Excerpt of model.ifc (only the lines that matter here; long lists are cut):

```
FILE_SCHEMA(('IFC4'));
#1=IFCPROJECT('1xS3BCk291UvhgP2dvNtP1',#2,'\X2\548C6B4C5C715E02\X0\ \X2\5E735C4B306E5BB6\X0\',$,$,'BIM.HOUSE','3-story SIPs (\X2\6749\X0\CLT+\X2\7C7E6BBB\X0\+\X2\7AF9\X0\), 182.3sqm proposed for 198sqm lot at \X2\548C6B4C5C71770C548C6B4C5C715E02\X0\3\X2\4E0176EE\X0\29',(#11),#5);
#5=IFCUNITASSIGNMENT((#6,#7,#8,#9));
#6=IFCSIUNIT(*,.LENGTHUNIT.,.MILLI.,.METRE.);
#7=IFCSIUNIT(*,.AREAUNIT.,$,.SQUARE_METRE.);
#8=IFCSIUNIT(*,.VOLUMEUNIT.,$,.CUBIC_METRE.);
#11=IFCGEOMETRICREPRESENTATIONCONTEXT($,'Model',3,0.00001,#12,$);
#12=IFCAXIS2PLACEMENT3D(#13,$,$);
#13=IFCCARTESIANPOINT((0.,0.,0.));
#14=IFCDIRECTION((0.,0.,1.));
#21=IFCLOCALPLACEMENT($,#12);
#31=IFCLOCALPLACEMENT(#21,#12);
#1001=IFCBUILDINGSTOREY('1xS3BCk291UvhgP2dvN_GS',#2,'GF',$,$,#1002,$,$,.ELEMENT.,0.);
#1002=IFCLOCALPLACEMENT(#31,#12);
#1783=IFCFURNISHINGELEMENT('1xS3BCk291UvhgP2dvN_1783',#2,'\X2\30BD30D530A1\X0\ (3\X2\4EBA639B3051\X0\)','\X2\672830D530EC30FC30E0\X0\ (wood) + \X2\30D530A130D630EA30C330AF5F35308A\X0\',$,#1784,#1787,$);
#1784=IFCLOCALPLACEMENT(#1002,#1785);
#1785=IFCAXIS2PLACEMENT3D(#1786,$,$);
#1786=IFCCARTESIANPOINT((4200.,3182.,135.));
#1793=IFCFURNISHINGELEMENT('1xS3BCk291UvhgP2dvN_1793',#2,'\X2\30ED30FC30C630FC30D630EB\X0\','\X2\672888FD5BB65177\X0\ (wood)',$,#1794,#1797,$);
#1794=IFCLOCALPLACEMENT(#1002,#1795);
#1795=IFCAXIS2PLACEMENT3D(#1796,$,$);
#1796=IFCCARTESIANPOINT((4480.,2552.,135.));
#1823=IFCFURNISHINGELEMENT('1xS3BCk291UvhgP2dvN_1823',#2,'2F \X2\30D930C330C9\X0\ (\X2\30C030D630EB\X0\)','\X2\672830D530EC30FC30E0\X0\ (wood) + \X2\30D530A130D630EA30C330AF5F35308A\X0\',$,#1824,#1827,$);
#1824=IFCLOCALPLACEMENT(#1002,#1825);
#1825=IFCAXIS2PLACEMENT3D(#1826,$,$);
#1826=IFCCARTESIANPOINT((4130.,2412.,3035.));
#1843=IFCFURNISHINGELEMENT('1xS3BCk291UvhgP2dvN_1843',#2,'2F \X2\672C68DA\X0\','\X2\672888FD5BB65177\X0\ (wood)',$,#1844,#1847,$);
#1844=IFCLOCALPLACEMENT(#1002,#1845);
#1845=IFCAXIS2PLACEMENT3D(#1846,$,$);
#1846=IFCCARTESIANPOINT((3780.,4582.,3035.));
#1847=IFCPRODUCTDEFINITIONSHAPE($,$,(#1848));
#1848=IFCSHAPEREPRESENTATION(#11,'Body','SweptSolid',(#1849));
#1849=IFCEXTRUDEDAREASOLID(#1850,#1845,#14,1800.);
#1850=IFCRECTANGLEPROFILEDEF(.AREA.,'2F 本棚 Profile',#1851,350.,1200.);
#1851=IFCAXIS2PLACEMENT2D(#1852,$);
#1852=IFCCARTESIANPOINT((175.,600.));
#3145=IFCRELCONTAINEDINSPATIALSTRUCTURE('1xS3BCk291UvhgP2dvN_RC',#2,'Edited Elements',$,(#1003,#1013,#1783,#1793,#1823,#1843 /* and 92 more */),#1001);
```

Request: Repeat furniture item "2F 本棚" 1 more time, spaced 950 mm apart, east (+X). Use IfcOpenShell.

```python
import numpy as np
import ifcopenshell
import ifcopenshell.api.geometry
import ifcopenshell.api.root
import ifcopenshell.util.element
import ifcopenshell.util.placement
import ifcopenshell.util.unit

model = ifcopenshell.open("model.ifc")
unit_scale = ifcopenshell.util.unit.calculate_unit_scale(model)


def reuse_history(source, copy):
    """copy_class also copies each property set's owner history, people and application; keep the originals."""
    for rel in copy.IsDefinedBy:
        if rel.is_a("IfcRelDefinesByProperties") and (history := rel.RelatingPropertyDefinition.OwnerHistory):
            rel.RelatingPropertyDefinition.OwnerHistory = source.OwnerHistory
            ifcopenshell.util.element.remove_deep2(model, history)


source = model.by_guid("1xS3BCk291UvhgP2dvN_1843")
base = ifcopenshell.util.placement.get_local_placement(source.ObjectPlacement)
step = np.array([1.0, 0.0, 0.0]) * 0.95 / unit_scale

for i in range(1, 2):
    copy = ifcopenshell.api.root.copy_class(model, product=source)
    copy.Representation = ifcopenshell.util.element.copy_deep(
        model, source.Representation, exclude=["IfcGeometricRepresentationContext", "IfcRepresentationMap"]
    )
    reuse_history(source, copy)
    matrix = base.copy()
    matrix[:3, 3] += i * step
    print("added at", matrix[:3, 3].round(3) + 0.0)
    ifcopenshell.api.geometry.edit_object_placement(model, product=copy, matrix=matrix, is_si=False)

model.write("model_v2.ifc")
```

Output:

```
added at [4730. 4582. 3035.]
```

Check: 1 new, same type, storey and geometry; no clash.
